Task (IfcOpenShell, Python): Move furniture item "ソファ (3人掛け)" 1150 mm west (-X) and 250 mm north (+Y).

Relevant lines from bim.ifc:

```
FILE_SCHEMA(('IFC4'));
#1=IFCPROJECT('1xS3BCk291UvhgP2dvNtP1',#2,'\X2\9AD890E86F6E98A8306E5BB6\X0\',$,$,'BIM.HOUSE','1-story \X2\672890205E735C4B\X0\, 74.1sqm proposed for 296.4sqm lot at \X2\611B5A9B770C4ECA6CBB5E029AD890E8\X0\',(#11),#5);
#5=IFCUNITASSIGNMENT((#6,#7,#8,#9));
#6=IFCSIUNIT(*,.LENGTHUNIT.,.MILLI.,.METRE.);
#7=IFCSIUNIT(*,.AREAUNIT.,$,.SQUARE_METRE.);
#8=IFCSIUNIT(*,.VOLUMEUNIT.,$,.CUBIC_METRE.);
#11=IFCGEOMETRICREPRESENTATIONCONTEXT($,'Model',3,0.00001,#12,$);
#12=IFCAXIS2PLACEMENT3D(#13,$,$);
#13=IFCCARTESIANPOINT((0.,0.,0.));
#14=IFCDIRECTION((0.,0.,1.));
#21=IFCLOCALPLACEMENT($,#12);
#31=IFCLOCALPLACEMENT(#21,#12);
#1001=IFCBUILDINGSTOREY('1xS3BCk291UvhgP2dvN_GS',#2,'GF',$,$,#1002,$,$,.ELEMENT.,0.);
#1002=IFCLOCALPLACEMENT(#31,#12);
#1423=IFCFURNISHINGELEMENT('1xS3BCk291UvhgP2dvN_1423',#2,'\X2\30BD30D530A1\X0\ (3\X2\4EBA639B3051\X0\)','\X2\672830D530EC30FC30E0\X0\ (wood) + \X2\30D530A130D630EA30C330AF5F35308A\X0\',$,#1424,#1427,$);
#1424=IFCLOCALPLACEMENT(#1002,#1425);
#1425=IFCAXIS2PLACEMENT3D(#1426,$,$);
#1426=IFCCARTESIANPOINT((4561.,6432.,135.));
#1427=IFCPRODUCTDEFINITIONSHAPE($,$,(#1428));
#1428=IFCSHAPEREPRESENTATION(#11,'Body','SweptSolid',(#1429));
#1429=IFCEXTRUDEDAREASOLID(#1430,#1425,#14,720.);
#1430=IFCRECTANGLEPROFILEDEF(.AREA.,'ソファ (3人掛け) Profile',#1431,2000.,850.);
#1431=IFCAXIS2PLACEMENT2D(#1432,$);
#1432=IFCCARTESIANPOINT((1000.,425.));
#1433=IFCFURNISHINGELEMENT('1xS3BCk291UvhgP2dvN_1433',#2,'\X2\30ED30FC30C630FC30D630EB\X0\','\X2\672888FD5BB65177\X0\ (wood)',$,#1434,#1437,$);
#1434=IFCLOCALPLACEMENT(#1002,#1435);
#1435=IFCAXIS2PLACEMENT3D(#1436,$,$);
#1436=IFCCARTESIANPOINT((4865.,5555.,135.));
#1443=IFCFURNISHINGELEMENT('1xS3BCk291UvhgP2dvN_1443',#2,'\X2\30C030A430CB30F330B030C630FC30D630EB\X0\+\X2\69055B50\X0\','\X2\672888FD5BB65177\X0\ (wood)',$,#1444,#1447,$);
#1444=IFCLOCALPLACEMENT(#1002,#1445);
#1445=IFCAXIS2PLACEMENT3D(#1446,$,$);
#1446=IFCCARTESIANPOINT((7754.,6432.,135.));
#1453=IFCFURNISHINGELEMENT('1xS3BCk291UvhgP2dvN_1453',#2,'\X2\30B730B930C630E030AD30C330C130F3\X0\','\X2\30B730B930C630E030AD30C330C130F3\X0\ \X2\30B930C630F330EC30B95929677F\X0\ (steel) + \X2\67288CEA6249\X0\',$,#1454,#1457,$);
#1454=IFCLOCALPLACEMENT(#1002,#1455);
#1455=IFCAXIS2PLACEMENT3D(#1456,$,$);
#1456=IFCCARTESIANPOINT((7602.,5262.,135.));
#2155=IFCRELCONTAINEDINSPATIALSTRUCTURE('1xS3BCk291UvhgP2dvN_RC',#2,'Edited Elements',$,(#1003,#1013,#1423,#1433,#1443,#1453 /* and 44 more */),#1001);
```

```python
import ifcopenshell
import ifcopenshell.api.geometry
import ifcopenshell.util.placement
import ifcopenshell.util.unit

model = ifcopenshell.open("bim.ifc")
unit_scale = ifcopenshell.util.unit.calculate_unit_scale(model)

item = model.by_id(1423)
matrix = ifcopenshell.util.placement.get_local_placement(item.ObjectPlacement)
matrix[0, 3] -= 1.15 / unit_scale
matrix[1, 3] += 0.25 / unit_scale
ifcopenshell.api.geometry.edit_object_placement(model, product=item, matrix=matrix, is_si=False)

print(ifcopenshell.util.placement.get_local_placement(item.ObjectPlacement).round(3) + 0.0)

model.write("bim_v2.ifc")
```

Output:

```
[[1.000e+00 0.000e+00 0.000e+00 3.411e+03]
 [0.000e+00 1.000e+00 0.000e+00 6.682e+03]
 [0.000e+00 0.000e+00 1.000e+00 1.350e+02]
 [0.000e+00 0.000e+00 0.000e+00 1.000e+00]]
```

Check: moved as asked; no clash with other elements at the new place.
